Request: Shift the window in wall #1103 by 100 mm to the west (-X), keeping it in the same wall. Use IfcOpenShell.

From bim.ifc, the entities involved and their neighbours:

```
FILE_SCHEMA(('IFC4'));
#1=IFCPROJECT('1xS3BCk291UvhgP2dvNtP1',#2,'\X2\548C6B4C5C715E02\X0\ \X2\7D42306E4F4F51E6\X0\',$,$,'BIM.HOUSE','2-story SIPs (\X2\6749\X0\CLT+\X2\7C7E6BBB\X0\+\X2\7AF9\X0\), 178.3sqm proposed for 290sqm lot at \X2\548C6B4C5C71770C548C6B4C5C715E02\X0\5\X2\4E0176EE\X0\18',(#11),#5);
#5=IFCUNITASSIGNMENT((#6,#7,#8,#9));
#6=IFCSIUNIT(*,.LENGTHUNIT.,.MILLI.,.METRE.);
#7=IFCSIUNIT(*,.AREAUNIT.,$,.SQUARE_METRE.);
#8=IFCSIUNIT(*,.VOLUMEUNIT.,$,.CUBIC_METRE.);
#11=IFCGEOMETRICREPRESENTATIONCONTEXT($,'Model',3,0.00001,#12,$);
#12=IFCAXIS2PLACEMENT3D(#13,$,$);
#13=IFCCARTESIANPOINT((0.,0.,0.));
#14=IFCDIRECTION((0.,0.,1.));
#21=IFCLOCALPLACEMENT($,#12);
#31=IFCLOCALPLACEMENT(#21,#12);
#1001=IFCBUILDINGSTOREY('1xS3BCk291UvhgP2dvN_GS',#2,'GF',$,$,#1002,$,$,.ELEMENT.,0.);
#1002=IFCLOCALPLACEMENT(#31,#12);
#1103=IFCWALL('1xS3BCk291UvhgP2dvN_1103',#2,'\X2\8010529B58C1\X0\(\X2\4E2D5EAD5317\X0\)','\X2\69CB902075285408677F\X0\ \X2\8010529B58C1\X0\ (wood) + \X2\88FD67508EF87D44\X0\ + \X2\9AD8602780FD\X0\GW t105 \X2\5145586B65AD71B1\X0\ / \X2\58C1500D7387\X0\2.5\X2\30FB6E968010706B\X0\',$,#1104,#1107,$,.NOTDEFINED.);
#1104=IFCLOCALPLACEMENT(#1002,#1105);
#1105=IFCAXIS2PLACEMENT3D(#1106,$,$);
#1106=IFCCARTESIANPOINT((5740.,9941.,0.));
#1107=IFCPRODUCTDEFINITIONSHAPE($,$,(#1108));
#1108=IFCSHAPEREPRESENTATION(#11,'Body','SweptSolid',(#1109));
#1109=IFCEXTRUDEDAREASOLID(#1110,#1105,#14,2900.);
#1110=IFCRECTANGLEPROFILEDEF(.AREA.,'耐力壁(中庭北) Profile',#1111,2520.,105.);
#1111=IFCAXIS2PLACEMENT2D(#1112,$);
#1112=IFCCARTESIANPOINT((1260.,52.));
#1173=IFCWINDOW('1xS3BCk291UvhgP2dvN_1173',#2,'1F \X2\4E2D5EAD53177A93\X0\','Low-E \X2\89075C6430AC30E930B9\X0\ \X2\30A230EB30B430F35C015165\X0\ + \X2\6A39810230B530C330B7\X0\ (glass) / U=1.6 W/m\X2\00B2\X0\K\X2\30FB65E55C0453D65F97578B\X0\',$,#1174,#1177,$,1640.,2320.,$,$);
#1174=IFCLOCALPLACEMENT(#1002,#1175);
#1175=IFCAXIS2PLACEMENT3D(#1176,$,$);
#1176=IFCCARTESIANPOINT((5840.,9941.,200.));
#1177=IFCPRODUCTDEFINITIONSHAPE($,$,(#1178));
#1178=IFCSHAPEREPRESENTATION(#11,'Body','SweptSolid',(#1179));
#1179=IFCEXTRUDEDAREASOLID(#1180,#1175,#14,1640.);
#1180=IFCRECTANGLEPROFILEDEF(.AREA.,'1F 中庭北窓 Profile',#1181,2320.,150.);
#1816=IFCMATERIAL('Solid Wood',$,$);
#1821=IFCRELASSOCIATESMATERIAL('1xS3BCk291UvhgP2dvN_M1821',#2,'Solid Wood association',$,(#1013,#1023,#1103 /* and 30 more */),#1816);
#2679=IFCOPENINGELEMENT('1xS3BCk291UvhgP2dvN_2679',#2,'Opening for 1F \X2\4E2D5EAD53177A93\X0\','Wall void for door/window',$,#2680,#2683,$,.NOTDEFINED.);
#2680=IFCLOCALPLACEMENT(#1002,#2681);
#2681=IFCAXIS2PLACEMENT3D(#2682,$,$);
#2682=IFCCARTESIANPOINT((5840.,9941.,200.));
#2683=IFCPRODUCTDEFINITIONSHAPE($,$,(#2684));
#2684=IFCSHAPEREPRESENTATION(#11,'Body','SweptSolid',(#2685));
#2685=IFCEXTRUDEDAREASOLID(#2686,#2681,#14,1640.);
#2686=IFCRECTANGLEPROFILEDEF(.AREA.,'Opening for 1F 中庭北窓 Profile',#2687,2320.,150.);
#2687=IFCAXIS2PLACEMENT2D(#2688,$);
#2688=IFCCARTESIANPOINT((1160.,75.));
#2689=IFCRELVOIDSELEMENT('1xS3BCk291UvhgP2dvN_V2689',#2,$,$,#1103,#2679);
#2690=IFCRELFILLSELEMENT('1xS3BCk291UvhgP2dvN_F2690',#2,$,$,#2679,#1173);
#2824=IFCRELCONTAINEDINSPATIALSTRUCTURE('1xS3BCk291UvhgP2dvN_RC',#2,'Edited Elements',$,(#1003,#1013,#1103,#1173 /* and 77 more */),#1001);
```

```python
import ifcopenshell
import ifcopenshell.api.geometry
import ifcopenshell.util.placement
import ifcopenshell.util.unit

model = ifcopenshell.open("bim.ifc")
unit_scale = ifcopenshell.util.unit.calculate_unit_scale(model)

window = model.by_id(1173)
opening = window.FillsVoids[0].RelatingOpeningElement
wall = opening.VoidsElements[0].RelatingBuildingElement

wall_matrix = ifcopenshell.util.placement.get_local_placement(wall.ObjectPlacement)
shift = wall_matrix[:3, 0] * -0.1 / unit_scale
before = ifcopenshell.util.placement.get_local_placement(window.ObjectPlacement)[:3, 3].copy()

# The window is not placed relative to its opening, so move both.
for product in (opening, window):
    matrix = ifcopenshell.util.placement.get_local_placement(product.ObjectPlacement)
    matrix[:3, 3] += shift
    ifcopenshell.api.geometry.edit_object_placement(model, product=product, matrix=matrix, is_si=False)

after = ifcopenshell.util.placement.get_local_placement(window.ObjectPlacement)[:3, 3]
print("window moved by", (after - before).round(3) + 0.0)

model.write("bim_edited.ifc")
```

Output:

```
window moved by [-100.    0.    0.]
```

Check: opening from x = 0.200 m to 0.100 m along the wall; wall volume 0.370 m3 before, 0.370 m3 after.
